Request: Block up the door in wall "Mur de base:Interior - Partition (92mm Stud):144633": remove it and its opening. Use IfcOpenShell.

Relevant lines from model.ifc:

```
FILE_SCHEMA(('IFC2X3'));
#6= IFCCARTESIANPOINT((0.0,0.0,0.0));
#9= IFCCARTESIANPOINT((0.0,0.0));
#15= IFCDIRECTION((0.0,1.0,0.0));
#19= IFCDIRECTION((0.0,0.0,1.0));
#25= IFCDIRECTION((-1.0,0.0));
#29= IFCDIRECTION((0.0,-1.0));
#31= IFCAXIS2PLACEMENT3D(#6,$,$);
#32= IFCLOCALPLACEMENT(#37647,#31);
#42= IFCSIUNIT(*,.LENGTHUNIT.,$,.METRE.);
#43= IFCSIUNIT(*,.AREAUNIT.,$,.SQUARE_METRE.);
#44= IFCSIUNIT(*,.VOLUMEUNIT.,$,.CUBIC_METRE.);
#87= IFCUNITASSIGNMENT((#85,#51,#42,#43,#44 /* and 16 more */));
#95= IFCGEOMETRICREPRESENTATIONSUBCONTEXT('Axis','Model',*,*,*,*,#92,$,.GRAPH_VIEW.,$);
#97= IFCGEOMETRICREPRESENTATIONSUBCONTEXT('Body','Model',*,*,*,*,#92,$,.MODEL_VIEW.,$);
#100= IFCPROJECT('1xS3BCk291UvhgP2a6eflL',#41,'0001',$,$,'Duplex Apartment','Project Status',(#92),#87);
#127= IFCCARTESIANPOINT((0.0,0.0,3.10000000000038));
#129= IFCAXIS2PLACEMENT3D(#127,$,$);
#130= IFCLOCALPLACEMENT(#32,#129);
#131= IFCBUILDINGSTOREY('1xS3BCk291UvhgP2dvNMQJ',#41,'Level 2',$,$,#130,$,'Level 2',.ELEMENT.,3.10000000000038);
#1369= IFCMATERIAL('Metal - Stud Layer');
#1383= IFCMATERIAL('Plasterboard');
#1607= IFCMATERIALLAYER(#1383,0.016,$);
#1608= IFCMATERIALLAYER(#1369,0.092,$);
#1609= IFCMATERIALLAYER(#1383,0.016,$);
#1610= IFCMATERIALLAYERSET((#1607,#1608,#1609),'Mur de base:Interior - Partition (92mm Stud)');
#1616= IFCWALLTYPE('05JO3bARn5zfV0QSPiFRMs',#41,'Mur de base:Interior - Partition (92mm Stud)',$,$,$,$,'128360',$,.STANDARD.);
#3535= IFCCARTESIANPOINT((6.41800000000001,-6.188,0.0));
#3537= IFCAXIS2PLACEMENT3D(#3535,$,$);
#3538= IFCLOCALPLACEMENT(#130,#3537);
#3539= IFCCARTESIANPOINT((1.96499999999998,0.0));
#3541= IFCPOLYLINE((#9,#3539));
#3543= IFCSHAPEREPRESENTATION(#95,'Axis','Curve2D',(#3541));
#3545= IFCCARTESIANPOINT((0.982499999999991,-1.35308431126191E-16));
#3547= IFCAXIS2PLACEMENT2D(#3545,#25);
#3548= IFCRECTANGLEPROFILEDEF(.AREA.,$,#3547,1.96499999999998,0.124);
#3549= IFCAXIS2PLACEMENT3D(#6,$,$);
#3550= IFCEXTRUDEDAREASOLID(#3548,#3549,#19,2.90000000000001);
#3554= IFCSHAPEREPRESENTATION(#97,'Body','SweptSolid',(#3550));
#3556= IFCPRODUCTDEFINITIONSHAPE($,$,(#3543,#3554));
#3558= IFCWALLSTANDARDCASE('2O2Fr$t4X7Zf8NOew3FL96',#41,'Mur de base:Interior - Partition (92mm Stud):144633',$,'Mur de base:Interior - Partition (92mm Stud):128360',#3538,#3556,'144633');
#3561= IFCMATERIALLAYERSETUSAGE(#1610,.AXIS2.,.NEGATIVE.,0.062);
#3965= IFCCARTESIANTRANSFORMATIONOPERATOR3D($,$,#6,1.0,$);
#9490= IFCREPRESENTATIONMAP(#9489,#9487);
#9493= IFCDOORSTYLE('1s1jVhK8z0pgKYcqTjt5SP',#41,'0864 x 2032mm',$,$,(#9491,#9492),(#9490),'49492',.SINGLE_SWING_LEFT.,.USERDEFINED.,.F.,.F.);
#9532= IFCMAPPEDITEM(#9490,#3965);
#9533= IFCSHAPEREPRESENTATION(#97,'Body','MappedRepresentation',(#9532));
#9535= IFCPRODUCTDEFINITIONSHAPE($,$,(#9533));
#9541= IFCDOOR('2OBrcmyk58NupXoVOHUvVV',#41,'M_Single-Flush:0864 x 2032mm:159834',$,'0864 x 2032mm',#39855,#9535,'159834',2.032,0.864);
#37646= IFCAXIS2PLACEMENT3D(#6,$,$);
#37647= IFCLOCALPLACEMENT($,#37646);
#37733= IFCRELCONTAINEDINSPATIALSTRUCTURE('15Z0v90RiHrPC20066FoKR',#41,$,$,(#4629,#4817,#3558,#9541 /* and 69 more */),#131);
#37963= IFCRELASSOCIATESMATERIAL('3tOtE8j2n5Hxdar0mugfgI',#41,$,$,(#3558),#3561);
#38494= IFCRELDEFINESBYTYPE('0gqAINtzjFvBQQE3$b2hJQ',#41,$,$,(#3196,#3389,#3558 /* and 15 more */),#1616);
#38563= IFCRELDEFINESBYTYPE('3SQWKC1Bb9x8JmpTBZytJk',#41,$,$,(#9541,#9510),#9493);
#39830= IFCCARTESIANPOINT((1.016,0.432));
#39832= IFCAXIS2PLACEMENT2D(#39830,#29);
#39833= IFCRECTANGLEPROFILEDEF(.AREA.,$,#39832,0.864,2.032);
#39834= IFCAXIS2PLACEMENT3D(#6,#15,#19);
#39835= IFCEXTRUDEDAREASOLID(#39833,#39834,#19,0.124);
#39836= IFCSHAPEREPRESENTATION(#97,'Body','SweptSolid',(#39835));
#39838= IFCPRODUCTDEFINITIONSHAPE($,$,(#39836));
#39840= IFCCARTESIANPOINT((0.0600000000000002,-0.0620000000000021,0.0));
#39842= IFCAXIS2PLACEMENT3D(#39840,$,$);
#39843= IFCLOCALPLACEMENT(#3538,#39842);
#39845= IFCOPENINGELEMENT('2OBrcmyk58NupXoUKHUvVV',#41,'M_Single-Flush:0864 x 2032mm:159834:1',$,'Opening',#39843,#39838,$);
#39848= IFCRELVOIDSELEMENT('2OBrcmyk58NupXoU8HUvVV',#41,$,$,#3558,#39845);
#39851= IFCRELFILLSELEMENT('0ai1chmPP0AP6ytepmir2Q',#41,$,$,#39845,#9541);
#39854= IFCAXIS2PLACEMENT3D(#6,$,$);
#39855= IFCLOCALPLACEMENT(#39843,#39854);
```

```python
import ifcopenshell
import ifcopenshell.api.feature
import ifcopenshell.api.root
import ifcopenshell.geom
import ifcopenshell.util.shape

model = ifcopenshell.open("model.ifc")
settings = ifcopenshell.geom.settings()


def volume(element):
    """Net volume in cubic metres, openings subtracted."""
    shape = ifcopenshell.geom.create_shape(settings, element)
    return ifcopenshell.util.shape.get_volume(shape.geometry)


door = model.by_guid("2OBrcmyk58NupXoVOHUvVV")
opening = door.FillsVoids[0].RelatingOpeningElement
wall = opening.VoidsElements[0].RelatingBuildingElement
before = volume(wall)

ifcopenshell.api.root.remove_product(model, product=door)
ifcopenshell.api.feature.remove_feature(model, feature=opening)

after = volume(wall)

print(f"wall volume {before:.3f} -> {after:.3f} m3")

model.write("model_updated.ifc")
```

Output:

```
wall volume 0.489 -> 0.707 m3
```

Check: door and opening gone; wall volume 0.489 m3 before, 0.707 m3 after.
